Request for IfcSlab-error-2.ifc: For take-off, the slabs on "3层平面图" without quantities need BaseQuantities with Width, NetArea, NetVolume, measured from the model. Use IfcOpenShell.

First a look at what the model holds.

```python
import ifcopenshell
import ifcopenshell.util.element
import ifcopenshell.util.unit

model = ifcopenshell.open("IfcSlab-error-2.ifc")
print(model.schema)
for unit_type in ("LENGTHUNIT", "AREAUNIT", "VOLUMEUNIT"):
    print(unit_type, ifcopenshell.util.unit.calculate_unit_scale(model, unit_type))
storey = next(s for s in model.by_type("IfcBuildingStorey") if s.Name == "3层平面图")
slabs = [e for e in ifcopenshell.util.element.get_decomposition(storey) if e.is_a("IfcSlab")]
for e in sorted(slabs, key=lambda e: e.id()):
    print(e.id(), e.is_a(), e.Name, list(ifcopenshell.util.element.get_psets(e, qtos_only=True)), sep=" | ")
```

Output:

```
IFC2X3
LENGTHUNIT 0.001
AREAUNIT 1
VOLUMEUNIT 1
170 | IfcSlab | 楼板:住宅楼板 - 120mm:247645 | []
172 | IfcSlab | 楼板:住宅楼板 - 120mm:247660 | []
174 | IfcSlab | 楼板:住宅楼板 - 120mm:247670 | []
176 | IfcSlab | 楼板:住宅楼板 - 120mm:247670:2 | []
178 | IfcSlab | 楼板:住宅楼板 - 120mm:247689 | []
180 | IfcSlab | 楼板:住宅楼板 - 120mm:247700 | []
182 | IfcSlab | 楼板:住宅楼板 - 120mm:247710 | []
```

```python
import ifcopenshell
import ifcopenshell.api.pset
import ifcopenshell.geom
import ifcopenshell.util.element
import ifcopenshell.util.shape
import ifcopenshell.util.unit

model = ifcopenshell.open("IfcSlab-error-2.ifc")
unit_scale = ifcopenshell.util.unit.calculate_unit_scale(model)
area_scale = ifcopenshell.util.unit.calculate_unit_scale(model, "AREAUNIT")
volume_scale = ifcopenshell.util.unit.calculate_unit_scale(model, "VOLUMEUNIT")
settings = ifcopenshell.geom.settings()

storey = next(s for s in model.by_type("IfcBuildingStorey") if s.Name == "3层平面图")
slabs = [e for e in ifcopenshell.util.element.get_decomposition(storey) if e.is_a("IfcSlab")]

for e in sorted(slabs, key=lambda e: e.id()):
    if ifcopenshell.util.element.get_psets(e, qtos_only=True, should_inherit=False):
        continue
    # Geometry comes back in metres, in the element's own axes.
    shape = ifcopenshell.geom.create_shape(settings, e)
    values = {
        "Width": ifcopenshell.util.shape.get_z(shape.geometry) / unit_scale,
        "NetArea": ifcopenshell.util.shape.get_footprint_area(shape.geometry) / area_scale,
        "NetVolume": ifcopenshell.util.shape.get_volume(shape.geometry) / volume_scale,
    }
    qto = ifcopenshell.api.pset.add_qto(model, product=e, name="BaseQuantities")
    ifcopenshell.api.pset.edit_qto(model, qto=qto, properties=values)
    print(e.id(), {k: round(v, 3) for k, v in values.items()})

model.write("IfcSlab-error-2_v2.ifc")
```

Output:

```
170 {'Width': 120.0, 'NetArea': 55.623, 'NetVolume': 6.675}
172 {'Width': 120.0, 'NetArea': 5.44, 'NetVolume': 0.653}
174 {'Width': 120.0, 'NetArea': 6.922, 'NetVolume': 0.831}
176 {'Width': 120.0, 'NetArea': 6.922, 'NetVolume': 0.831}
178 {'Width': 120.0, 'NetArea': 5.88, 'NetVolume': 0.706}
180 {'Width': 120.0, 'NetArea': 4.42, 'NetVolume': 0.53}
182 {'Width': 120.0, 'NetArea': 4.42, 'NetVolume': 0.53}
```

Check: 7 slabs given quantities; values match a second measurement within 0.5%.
